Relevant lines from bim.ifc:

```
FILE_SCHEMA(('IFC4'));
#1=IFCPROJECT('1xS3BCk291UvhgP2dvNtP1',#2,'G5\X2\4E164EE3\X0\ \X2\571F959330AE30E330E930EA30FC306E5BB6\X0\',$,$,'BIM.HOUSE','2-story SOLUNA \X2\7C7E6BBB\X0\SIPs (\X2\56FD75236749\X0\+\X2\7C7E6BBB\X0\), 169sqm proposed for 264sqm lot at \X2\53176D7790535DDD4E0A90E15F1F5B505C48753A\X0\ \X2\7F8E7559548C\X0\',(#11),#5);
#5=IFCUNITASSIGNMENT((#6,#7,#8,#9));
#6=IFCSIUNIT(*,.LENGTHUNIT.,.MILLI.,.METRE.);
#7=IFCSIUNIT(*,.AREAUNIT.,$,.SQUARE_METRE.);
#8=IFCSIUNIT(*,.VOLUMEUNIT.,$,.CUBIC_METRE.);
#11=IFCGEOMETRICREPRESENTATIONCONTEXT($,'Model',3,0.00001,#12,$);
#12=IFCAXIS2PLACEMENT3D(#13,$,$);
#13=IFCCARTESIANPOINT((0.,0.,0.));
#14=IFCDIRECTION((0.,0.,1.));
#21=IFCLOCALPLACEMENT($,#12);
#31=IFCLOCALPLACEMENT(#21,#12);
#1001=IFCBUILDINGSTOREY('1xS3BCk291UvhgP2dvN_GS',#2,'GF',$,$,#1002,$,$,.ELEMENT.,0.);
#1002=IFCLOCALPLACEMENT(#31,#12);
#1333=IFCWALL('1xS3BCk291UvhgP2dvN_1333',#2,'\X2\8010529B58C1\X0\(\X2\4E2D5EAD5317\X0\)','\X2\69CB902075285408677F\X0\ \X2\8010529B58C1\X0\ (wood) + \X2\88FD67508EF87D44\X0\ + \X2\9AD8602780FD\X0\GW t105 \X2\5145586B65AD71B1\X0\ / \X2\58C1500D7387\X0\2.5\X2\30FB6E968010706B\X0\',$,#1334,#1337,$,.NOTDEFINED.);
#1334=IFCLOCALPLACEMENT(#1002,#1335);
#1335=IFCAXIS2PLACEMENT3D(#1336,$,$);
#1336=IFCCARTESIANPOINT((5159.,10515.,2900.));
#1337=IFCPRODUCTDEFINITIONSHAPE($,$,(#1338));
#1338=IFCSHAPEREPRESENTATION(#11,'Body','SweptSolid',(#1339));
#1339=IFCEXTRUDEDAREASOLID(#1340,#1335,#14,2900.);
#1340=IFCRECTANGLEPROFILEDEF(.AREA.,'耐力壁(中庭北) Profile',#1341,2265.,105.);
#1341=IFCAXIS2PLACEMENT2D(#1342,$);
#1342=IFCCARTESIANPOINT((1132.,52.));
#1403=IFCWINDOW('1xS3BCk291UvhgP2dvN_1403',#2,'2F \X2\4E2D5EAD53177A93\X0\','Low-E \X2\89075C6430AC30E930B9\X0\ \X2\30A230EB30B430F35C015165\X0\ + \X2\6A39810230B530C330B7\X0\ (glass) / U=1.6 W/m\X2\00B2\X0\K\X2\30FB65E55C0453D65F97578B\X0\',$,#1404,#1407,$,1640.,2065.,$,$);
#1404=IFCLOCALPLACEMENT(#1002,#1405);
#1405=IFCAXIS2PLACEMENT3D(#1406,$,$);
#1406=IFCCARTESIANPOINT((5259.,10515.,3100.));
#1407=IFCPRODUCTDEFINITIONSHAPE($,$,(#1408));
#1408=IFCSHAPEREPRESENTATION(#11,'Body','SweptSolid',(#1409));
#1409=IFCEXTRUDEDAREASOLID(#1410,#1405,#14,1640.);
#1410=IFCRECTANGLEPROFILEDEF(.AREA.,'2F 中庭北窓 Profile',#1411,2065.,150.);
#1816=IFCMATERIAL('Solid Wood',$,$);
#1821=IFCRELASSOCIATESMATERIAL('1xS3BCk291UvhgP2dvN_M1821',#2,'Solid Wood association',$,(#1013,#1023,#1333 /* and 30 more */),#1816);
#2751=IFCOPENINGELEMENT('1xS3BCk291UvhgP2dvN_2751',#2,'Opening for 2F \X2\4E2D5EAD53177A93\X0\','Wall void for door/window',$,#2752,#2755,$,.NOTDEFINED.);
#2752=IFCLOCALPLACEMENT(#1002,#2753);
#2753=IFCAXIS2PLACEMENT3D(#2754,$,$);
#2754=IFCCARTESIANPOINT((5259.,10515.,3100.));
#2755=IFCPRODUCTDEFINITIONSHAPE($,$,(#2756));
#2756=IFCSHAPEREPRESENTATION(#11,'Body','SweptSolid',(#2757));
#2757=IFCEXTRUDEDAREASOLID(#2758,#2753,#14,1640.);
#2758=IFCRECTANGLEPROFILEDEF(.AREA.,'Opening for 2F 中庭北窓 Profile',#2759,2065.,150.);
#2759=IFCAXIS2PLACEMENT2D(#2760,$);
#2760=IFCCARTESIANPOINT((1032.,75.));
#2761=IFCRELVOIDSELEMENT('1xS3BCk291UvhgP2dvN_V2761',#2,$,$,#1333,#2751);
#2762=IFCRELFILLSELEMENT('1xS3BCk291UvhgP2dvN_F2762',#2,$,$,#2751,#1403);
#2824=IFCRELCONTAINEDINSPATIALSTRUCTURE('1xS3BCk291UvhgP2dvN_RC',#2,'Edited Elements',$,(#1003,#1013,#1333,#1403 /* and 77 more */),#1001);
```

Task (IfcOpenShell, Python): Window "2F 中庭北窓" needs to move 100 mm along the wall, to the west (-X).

```python
import ifcopenshell
import ifcopenshell.api.geometry
import ifcopenshell.util.placement
import ifcopenshell.util.unit

model = ifcopenshell.open("bim.ifc")
unit_scale = ifcopenshell.util.unit.calculate_unit_scale(model)

window = model.by_guid("1xS3BCk291UvhgP2dvN_1403")
opening = window.FillsVoids[0].RelatingOpeningElement
wall = opening.VoidsElements[0].RelatingBuildingElement

wall_matrix = ifcopenshell.util.placement.get_local_placement(wall.ObjectPlacement)
shift = wall_matrix[:3, 0] * -0.1 / unit_scale
before = ifcopenshell.util.placement.get_local_placement(window.ObjectPlacement)[:3, 3].copy()

# The window is not placed relative to its opening, so move both.
for product in (opening, window):
    matrix = ifcopenshell.util.placement.get_local_placement(product.ObjectPlacement)
    matrix[:3, 3] += shift
    ifcopenshell.api.geometry.edit_object_placement(model, product=product, matrix=matrix, is_si=False)

after = ifcopenshell.util.placement.get_local_placement(window.ObjectPlacement)[:3, 3]
print("window moved by", (after - before).round(3) + 0.0)

model.write("bim_rev.ifc")
```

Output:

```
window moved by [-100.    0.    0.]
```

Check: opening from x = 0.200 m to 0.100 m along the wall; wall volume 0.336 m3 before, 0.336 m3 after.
